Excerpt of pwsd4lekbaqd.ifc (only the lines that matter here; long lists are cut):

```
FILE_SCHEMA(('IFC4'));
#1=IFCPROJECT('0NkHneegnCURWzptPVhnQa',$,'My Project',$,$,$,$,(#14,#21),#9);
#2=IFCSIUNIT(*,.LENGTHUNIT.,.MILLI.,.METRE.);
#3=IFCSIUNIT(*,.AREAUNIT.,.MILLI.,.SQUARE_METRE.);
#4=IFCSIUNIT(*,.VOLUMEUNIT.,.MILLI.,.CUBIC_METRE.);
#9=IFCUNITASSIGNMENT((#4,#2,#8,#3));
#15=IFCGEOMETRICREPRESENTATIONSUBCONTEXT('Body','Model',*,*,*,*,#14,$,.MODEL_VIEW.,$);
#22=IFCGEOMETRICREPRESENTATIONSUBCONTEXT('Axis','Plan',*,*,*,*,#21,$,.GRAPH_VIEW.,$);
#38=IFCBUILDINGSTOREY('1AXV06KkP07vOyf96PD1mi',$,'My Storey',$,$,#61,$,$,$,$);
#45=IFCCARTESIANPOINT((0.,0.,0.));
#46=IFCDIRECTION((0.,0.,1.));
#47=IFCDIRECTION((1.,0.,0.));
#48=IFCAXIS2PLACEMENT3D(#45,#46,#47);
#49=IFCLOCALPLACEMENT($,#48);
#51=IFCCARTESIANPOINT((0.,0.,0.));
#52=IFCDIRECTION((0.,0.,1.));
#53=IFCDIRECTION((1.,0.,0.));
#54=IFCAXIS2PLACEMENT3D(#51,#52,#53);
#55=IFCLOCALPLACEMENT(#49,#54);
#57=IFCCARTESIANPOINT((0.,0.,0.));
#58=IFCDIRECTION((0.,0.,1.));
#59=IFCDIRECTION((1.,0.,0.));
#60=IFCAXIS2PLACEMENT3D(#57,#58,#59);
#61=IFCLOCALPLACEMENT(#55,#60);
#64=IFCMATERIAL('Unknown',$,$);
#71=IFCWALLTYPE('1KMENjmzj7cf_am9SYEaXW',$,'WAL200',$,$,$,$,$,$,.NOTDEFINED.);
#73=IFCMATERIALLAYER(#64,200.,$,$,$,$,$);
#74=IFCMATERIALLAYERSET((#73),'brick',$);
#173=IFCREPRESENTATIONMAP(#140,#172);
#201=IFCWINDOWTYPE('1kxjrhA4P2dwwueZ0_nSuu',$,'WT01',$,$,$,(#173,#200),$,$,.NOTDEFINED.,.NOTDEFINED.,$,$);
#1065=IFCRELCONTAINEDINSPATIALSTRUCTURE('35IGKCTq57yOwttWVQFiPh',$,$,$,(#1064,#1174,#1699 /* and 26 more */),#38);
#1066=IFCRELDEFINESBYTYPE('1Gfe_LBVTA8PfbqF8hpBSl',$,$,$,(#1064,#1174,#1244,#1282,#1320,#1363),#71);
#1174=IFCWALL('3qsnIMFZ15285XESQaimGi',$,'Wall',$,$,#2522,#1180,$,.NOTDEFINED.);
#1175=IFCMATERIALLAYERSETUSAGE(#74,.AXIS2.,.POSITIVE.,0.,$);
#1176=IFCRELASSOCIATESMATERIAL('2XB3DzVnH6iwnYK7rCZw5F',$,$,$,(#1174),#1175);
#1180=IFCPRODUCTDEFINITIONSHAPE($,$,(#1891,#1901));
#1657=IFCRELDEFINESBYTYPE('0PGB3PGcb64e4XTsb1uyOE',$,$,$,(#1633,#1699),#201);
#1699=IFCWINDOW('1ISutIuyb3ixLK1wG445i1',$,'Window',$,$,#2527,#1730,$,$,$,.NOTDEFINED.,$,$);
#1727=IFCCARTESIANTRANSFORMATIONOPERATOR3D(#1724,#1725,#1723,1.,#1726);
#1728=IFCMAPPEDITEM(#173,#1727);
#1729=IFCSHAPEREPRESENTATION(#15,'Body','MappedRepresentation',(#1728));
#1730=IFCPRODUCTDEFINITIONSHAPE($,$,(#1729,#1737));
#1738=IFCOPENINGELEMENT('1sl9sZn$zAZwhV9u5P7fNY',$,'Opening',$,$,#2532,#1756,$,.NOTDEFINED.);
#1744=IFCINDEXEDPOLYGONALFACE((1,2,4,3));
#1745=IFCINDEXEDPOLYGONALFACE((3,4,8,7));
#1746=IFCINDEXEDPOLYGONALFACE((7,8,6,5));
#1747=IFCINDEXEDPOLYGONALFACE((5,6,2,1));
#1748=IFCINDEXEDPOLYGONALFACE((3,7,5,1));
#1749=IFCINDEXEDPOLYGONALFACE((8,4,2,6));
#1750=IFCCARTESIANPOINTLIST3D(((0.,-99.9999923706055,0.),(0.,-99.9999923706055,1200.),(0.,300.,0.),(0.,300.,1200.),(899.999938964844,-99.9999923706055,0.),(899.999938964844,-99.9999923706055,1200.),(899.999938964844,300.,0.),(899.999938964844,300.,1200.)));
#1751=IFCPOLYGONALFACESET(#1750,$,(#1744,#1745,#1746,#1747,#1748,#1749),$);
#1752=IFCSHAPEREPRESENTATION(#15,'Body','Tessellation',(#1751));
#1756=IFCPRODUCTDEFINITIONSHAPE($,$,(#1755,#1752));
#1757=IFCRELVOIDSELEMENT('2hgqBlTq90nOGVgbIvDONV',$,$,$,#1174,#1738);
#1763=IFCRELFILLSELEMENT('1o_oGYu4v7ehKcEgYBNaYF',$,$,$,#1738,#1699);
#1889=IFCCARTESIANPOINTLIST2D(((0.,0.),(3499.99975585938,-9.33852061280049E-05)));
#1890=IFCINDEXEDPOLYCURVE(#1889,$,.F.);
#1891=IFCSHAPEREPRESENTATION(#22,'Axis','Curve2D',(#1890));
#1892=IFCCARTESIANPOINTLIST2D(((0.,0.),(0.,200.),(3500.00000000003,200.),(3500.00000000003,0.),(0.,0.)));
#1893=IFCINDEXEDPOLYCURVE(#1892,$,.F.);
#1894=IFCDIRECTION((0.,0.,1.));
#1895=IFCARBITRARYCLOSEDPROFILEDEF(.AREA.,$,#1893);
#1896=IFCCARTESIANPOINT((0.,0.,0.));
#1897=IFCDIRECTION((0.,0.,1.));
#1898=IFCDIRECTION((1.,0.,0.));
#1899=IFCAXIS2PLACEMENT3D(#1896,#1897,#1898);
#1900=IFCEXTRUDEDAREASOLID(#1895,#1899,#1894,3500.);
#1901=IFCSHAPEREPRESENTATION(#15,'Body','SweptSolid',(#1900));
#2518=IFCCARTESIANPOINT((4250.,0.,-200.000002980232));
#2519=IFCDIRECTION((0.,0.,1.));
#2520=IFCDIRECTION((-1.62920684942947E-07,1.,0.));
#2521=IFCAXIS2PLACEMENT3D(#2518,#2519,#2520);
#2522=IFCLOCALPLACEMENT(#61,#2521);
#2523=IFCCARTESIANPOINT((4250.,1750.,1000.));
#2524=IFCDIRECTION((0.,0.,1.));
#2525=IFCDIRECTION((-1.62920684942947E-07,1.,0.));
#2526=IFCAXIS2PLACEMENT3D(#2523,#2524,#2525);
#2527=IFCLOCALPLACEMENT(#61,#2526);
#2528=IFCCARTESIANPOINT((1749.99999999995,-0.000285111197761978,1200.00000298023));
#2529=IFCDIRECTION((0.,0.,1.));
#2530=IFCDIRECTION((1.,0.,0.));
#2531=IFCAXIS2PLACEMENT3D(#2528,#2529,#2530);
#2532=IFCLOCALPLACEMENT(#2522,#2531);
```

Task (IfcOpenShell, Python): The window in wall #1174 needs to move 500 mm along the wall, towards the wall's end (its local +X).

```python
import ifcopenshell
import ifcopenshell.api.geometry
import ifcopenshell.util.placement
import ifcopenshell.util.unit

model = ifcopenshell.open("pwsd4lekbaqd.ifc")
unit_scale = ifcopenshell.util.unit.calculate_unit_scale(model)

window = model.by_guid("1ISutIuyb3ixLK1wG445i1")
opening = window.FillsVoids[0].RelatingOpeningElement
wall = opening.VoidsElements[0].RelatingBuildingElement

wall_matrix = ifcopenshell.util.placement.get_local_placement(wall.ObjectPlacement)
shift = wall_matrix[:3, 0] * 0.5 / unit_scale
before = ifcopenshell.util.placement.get_local_placement(window.ObjectPlacement)[:3, 3].copy()

# The window is not placed relative to its opening, so move both.
for product in (opening, window):
    matrix = ifcopenshell.util.placement.get_local_placement(product.ObjectPlacement)
    matrix[:3, 3] += shift
    ifcopenshell.api.geometry.edit_object_placement(model, product=product, matrix=matrix, is_si=False)

after = ifcopenshell.util.placement.get_local_placement(window.ObjectPlacement)[:3, 3]
print("window moved by", (after - before).round(3) + 0.0)

model.write("pwsd4lekbaqd-out.ifc")
```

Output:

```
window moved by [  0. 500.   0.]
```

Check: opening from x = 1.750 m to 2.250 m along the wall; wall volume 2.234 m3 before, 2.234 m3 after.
